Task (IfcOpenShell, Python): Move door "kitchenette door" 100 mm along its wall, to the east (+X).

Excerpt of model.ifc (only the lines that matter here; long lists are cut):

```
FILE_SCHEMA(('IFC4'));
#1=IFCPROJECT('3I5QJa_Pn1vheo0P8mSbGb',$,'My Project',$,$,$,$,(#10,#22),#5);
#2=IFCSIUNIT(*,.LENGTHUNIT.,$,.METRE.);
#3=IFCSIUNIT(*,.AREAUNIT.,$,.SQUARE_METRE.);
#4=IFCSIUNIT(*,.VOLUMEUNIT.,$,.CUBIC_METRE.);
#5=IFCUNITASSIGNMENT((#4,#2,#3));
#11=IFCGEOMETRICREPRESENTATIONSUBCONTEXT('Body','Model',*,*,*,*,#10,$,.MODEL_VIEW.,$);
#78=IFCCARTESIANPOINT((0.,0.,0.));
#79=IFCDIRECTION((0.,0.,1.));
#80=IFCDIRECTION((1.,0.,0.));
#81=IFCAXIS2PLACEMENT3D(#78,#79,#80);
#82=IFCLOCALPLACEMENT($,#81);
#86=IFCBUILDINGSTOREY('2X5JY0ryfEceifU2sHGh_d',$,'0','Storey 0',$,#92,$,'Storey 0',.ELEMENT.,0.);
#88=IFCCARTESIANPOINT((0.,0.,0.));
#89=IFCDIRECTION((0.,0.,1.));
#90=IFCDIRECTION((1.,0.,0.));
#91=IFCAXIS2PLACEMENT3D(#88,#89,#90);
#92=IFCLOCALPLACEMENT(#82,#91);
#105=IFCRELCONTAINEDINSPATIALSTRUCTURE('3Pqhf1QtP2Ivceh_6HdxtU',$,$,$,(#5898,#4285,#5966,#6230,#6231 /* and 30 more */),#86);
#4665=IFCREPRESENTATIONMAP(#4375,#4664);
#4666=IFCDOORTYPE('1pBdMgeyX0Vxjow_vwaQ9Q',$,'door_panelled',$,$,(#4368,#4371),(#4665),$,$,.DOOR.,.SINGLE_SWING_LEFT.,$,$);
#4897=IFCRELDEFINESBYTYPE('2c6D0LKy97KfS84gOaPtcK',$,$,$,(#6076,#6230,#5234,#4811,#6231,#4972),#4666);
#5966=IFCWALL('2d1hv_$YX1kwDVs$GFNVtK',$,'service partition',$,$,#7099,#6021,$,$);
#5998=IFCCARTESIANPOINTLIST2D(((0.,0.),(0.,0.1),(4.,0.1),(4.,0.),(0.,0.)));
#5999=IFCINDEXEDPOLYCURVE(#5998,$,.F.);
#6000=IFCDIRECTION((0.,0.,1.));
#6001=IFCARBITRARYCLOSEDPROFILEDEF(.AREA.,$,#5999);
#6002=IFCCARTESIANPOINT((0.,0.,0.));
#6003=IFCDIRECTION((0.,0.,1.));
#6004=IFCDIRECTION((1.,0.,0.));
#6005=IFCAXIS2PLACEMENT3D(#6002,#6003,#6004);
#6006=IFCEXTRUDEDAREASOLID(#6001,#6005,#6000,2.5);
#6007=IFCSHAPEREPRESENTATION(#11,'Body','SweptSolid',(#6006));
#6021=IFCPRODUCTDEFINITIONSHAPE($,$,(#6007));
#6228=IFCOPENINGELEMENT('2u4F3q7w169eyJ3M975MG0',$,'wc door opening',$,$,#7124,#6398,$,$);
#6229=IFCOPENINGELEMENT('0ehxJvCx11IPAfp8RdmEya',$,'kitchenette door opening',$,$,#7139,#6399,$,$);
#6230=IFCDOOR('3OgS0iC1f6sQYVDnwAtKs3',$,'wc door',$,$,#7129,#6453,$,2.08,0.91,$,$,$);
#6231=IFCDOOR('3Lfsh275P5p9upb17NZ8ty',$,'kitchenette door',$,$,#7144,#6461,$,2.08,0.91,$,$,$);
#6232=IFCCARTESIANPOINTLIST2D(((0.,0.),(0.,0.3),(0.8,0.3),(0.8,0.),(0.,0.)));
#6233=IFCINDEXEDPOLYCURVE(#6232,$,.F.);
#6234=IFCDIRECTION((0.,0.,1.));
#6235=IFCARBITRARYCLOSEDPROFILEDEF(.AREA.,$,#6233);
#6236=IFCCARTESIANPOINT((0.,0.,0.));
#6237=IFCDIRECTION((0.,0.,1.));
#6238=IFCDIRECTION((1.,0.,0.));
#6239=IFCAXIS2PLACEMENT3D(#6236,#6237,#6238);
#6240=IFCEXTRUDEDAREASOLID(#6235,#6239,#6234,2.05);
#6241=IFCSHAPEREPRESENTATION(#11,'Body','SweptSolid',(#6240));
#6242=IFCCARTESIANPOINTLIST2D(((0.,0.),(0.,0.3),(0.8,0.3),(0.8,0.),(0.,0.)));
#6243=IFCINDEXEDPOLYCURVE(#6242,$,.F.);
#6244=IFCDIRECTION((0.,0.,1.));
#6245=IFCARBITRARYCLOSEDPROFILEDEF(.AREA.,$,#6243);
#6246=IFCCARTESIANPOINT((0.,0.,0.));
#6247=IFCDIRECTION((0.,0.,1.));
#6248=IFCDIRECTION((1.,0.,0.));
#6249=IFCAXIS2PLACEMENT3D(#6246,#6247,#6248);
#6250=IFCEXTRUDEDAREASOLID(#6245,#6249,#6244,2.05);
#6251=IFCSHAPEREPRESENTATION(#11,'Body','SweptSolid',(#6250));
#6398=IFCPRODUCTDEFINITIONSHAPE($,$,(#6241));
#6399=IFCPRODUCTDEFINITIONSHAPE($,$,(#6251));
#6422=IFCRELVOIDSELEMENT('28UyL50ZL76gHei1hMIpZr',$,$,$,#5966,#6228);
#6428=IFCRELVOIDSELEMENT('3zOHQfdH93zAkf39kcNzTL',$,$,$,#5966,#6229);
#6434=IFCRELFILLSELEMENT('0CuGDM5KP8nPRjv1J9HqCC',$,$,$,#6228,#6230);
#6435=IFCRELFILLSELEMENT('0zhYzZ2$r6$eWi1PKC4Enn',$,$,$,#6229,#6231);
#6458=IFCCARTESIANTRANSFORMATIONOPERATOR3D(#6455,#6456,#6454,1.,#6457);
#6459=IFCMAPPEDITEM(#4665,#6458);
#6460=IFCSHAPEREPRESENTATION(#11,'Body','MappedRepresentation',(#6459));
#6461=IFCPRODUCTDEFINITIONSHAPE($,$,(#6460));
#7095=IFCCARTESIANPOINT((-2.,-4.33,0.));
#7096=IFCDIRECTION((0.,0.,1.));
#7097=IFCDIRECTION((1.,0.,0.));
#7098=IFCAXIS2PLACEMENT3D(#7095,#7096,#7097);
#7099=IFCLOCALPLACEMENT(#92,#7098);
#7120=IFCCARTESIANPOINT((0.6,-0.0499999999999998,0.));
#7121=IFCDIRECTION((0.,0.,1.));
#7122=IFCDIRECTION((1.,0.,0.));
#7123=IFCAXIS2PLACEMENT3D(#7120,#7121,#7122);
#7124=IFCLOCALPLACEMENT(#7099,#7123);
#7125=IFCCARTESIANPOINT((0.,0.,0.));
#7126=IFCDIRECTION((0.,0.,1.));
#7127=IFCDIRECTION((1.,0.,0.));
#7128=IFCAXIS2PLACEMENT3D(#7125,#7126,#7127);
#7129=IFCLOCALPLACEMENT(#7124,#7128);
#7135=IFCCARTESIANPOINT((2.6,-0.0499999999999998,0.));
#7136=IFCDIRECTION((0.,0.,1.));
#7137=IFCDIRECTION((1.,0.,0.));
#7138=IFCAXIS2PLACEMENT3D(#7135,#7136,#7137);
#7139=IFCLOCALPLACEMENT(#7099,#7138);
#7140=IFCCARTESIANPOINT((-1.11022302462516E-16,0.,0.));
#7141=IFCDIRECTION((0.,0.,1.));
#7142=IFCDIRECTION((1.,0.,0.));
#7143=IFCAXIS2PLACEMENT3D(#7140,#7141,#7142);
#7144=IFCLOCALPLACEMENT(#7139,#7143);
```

```python
import ifcopenshell
import ifcopenshell.api.geometry
import ifcopenshell.util.placement
import ifcopenshell.util.unit

model = ifcopenshell.open("model.ifc")
unit_scale = ifcopenshell.util.unit.calculate_unit_scale(model)

door = model.by_guid("3Lfsh275P5p9upb17NZ8ty")
opening = door.FillsVoids[0].RelatingOpeningElement
wall = opening.VoidsElements[0].RelatingBuildingElement

wall_matrix = ifcopenshell.util.placement.get_local_placement(wall.ObjectPlacement)
shift = wall_matrix[:3, 0] * 0.1 / unit_scale
before = ifcopenshell.util.placement.get_local_placement(door.ObjectPlacement)[:3, 3].copy()

# The door is placed relative to its opening, so it follows when the opening moves.
matrix = ifcopenshell.util.placement.get_local_placement(opening.ObjectPlacement)
matrix[:3, 3] += shift
ifcopenshell.api.geometry.edit_object_placement(
    model, product=opening, matrix=matrix, is_si=False, should_transform_children=True
)

after = ifcopenshell.util.placement.get_local_placement(door.ObjectPlacement)[:3, 3]
print("door moved by", (after - before).round(3) + 0.0)

model.write("model_edited.ifc")
```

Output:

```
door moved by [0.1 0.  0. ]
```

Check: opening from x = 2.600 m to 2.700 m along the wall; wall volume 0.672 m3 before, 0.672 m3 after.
